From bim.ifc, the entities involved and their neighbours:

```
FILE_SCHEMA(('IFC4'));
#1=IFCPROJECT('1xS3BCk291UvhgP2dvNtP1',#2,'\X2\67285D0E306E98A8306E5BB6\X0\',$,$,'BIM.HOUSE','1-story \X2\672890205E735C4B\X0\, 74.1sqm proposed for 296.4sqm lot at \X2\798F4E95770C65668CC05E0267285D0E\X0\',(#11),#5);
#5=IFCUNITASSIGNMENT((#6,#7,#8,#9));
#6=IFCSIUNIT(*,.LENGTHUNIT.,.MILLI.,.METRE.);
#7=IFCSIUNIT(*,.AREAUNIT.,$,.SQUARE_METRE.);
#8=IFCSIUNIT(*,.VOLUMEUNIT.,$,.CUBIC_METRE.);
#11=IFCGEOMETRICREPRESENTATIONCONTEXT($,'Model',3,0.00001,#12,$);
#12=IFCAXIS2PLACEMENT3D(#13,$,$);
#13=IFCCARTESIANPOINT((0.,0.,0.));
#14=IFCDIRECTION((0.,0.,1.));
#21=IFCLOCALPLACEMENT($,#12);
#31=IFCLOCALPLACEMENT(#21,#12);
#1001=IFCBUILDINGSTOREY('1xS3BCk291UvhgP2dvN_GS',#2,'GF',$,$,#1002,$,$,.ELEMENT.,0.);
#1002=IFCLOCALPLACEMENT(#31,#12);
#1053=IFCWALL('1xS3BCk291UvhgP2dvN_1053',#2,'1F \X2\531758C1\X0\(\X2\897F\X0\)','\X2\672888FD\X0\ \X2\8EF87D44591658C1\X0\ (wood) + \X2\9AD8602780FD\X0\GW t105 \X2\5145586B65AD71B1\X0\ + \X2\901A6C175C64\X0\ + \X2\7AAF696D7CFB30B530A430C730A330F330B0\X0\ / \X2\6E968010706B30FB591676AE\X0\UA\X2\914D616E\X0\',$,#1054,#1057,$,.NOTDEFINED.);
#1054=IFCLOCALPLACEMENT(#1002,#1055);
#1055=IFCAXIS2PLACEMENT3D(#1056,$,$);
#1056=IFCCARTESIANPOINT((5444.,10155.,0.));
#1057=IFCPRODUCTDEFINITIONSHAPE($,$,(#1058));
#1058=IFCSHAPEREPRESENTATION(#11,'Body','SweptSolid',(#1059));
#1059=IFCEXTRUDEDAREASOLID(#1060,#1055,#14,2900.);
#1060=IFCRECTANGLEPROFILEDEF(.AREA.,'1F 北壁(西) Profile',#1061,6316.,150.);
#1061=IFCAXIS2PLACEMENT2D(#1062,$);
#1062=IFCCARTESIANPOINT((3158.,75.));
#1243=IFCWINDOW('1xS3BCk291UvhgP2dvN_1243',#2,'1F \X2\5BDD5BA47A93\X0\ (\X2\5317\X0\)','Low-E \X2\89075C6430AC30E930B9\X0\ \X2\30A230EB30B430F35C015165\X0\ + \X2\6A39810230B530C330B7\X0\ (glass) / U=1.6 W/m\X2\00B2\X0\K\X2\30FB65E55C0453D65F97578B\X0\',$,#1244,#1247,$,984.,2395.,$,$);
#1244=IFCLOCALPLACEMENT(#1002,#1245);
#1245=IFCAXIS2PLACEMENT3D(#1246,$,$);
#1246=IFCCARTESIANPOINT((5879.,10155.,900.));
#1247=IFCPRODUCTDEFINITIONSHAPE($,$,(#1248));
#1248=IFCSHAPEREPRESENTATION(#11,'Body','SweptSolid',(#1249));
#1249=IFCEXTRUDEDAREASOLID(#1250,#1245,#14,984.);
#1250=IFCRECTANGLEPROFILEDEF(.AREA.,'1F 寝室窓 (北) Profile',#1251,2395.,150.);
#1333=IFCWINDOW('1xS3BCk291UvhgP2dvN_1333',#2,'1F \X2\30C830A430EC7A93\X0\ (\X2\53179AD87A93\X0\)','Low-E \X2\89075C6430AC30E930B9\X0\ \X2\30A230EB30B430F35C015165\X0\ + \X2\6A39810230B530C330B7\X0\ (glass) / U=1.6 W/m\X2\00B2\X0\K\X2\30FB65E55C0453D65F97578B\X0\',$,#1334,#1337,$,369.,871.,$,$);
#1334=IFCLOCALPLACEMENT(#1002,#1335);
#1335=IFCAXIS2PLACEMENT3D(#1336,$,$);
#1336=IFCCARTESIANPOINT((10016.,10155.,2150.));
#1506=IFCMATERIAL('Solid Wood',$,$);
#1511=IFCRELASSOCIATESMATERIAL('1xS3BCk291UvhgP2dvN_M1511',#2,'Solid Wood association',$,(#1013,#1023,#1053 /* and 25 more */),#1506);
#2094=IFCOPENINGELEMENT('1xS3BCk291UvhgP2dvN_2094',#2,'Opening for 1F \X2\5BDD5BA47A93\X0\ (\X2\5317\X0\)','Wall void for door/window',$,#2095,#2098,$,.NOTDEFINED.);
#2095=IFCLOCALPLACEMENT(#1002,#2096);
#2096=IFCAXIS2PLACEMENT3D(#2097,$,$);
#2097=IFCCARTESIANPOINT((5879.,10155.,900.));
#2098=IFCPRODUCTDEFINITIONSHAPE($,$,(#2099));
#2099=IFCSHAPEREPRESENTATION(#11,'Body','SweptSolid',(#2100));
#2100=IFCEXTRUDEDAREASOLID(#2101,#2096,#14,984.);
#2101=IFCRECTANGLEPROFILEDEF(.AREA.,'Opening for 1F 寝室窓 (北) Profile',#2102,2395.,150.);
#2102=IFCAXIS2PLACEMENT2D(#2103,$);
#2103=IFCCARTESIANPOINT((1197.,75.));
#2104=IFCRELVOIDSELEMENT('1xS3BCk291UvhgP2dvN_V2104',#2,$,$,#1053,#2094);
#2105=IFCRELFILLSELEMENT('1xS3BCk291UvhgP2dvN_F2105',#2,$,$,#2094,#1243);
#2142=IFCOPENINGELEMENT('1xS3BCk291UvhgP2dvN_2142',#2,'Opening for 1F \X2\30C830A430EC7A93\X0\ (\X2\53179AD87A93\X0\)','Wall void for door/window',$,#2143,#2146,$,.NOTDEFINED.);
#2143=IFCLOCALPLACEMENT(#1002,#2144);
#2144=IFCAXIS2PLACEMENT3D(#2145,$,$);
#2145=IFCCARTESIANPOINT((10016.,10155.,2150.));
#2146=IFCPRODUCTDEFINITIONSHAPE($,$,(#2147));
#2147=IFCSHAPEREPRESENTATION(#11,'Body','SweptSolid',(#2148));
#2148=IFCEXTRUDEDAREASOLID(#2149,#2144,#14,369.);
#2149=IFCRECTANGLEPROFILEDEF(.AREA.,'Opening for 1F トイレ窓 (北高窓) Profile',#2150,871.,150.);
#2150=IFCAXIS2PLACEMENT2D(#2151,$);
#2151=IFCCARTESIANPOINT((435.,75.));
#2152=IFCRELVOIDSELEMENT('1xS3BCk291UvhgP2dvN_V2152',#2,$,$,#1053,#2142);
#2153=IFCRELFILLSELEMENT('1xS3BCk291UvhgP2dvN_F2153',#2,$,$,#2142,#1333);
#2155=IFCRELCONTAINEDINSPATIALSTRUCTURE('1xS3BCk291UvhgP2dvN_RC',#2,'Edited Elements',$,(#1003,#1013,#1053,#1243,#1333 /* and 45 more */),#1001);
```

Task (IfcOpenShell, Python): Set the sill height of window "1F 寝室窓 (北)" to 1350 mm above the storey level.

```python
import numpy as np
import ifcopenshell
import ifcopenshell.api.geometry
import ifcopenshell.geom
import ifcopenshell.util.element
import ifcopenshell.util.placement
import ifcopenshell.util.shape
import ifcopenshell.util.unit

model = ifcopenshell.open("bim.ifc")
unit_scale = ifcopenshell.util.unit.calculate_unit_scale(model)

window = model.by_guid("1xS3BCk291UvhgP2dvN_1243")
opening = window.FillsVoids[0].RelatingOpeningElement
storey = ifcopenshell.util.element.get_container(window, ifc_class="IfcBuildingStorey")
level = ifcopenshell.util.placement.get_local_placement(storey.ObjectPlacement)[2, 3]

# The opening's origin need not be at the sill, so measure its lowest point.
shape = ifcopenshell.geom.create_shape(ifcopenshell.geom.settings(), opening)
bottom = ifcopenshell.util.shape.get_shape_bottom_elevation(shape, shape.geometry) / unit_scale
dz = level + 1350.0 - bottom

shift = np.array([0.0, 0.0, dz])
# The window is not placed relative to its opening, so move both.
for product in (opening, window):
    matrix = ifcopenshell.util.placement.get_local_placement(product.ObjectPlacement)
    matrix[:3, 3] += shift
    ifcopenshell.api.geometry.edit_object_placement(model, product=product, matrix=matrix, is_si=False)

print(f"moved by {dz * unit_scale:+.3f} m")

model.write("bim_v2.ifc")
```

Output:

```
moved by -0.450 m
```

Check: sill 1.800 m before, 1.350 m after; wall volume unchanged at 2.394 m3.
